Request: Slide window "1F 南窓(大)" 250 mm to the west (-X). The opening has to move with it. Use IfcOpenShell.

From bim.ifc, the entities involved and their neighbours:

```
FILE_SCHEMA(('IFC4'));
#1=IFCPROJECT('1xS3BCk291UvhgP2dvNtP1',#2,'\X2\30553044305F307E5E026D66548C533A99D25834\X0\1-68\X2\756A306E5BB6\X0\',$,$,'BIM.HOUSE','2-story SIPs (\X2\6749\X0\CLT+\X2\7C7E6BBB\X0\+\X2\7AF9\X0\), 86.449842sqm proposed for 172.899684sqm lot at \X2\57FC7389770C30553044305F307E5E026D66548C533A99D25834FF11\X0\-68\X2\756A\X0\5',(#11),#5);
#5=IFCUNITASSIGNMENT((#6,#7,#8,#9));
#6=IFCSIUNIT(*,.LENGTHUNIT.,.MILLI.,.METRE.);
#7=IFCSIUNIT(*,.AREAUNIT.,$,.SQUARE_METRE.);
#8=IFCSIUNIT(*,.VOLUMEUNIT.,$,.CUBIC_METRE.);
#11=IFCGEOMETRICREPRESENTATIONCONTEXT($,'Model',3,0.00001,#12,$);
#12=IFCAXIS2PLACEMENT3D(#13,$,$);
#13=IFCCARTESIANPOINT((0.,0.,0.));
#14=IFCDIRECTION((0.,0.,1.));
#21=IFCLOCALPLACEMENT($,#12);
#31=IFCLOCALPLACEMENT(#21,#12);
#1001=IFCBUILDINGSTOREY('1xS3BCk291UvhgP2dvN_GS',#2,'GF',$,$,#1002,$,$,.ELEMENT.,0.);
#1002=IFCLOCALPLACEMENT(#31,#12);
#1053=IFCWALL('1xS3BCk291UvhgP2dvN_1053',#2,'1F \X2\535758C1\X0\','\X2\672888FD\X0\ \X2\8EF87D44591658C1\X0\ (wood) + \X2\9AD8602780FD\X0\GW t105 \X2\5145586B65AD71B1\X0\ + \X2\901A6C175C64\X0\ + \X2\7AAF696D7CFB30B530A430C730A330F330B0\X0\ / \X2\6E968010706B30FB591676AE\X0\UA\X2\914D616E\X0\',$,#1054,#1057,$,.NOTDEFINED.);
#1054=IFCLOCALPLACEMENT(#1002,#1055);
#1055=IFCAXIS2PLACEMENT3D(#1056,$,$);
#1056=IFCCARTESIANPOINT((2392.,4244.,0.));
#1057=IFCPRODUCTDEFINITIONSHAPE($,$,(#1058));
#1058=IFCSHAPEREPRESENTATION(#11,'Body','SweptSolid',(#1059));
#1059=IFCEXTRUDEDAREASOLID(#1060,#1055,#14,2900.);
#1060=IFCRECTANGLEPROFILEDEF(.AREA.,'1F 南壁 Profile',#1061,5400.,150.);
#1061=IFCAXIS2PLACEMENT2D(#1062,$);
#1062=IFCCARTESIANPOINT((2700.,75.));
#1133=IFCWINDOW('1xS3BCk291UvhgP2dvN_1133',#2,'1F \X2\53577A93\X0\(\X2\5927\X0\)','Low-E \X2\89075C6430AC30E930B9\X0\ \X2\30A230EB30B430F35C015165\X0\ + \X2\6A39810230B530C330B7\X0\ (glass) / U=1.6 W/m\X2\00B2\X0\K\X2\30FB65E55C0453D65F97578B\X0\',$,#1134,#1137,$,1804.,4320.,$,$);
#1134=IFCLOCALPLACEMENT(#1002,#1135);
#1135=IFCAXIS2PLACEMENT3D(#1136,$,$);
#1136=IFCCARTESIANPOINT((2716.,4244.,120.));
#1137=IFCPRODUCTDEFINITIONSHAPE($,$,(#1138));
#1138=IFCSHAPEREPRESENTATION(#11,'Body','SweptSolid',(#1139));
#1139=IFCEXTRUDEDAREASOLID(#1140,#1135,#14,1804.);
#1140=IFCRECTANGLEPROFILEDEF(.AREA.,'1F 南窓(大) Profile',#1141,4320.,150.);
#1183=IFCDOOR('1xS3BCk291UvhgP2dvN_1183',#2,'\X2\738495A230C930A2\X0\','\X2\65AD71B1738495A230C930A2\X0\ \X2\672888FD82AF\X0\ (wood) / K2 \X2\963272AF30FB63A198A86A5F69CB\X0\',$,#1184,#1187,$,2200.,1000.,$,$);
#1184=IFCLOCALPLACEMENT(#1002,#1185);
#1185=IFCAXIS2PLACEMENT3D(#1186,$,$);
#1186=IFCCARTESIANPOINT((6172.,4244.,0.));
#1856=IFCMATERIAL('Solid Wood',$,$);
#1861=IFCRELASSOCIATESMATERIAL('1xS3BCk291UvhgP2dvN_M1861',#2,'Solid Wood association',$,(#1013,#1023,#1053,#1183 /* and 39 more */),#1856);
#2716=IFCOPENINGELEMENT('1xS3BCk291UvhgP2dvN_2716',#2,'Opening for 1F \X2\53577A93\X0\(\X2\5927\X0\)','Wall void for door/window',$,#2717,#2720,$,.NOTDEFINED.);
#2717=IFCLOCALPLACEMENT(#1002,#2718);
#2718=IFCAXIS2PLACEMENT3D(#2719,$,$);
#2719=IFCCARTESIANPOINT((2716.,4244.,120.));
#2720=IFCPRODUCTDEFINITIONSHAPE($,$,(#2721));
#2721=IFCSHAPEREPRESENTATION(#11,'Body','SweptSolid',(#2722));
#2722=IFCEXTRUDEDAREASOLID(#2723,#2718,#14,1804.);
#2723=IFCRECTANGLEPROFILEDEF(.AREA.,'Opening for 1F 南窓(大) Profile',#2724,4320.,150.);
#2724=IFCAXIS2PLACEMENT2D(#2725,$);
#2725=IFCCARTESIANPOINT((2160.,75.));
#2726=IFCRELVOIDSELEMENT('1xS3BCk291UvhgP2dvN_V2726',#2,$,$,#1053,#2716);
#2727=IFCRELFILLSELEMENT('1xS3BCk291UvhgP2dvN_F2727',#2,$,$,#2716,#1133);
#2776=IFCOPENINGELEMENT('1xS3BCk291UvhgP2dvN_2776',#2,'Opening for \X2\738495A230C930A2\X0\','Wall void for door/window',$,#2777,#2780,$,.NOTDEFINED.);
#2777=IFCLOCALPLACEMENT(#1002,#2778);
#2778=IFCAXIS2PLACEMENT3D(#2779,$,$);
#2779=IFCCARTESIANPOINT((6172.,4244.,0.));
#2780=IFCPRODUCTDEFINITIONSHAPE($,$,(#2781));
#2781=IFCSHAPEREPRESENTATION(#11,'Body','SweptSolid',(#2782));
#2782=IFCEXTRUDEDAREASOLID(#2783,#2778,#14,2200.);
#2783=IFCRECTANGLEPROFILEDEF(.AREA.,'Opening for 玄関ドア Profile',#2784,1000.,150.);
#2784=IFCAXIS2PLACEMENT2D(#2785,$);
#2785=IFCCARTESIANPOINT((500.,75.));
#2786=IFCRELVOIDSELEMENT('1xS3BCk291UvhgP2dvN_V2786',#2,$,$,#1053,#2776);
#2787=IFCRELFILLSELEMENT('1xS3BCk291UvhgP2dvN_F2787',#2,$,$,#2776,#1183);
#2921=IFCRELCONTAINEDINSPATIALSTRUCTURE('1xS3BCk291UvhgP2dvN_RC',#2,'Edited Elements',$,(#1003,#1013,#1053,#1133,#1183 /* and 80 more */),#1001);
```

```python
import ifcopenshell
import ifcopenshell.api.geometry
import ifcopenshell.util.placement
import ifcopenshell.util.unit

model = ifcopenshell.open("bim.ifc")
unit_scale = ifcopenshell.util.unit.calculate_unit_scale(model)

window = model.by_guid("1xS3BCk291UvhgP2dvN_1133")
opening = window.FillsVoids[0].RelatingOpeningElement
wall = opening.VoidsElements[0].RelatingBuildingElement

wall_matrix = ifcopenshell.util.placement.get_local_placement(wall.ObjectPlacement)
shift = wall_matrix[:3, 0] * -0.25 / unit_scale
before = ifcopenshell.util.placement.get_local_placement(window.ObjectPlacement)[:3, 3].copy()

# The window is not placed relative to its opening, so move both.
for product in (opening, window):
    matrix = ifcopenshell.util.placement.get_local_placement(product.ObjectPlacement)
    matrix[:3, 3] += shift
    ifcopenshell.api.geometry.edit_object_placement(model, product=product, matrix=matrix, is_si=False)

after = ifcopenshell.util.placement.get_local_placement(window.ObjectPlacement)[:3, 3]
print("window moved by", (after - before).round(3) + 0.0)

model.write("bim-out.ifc")
```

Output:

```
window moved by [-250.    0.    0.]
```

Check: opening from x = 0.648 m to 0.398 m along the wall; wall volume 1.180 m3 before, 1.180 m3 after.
